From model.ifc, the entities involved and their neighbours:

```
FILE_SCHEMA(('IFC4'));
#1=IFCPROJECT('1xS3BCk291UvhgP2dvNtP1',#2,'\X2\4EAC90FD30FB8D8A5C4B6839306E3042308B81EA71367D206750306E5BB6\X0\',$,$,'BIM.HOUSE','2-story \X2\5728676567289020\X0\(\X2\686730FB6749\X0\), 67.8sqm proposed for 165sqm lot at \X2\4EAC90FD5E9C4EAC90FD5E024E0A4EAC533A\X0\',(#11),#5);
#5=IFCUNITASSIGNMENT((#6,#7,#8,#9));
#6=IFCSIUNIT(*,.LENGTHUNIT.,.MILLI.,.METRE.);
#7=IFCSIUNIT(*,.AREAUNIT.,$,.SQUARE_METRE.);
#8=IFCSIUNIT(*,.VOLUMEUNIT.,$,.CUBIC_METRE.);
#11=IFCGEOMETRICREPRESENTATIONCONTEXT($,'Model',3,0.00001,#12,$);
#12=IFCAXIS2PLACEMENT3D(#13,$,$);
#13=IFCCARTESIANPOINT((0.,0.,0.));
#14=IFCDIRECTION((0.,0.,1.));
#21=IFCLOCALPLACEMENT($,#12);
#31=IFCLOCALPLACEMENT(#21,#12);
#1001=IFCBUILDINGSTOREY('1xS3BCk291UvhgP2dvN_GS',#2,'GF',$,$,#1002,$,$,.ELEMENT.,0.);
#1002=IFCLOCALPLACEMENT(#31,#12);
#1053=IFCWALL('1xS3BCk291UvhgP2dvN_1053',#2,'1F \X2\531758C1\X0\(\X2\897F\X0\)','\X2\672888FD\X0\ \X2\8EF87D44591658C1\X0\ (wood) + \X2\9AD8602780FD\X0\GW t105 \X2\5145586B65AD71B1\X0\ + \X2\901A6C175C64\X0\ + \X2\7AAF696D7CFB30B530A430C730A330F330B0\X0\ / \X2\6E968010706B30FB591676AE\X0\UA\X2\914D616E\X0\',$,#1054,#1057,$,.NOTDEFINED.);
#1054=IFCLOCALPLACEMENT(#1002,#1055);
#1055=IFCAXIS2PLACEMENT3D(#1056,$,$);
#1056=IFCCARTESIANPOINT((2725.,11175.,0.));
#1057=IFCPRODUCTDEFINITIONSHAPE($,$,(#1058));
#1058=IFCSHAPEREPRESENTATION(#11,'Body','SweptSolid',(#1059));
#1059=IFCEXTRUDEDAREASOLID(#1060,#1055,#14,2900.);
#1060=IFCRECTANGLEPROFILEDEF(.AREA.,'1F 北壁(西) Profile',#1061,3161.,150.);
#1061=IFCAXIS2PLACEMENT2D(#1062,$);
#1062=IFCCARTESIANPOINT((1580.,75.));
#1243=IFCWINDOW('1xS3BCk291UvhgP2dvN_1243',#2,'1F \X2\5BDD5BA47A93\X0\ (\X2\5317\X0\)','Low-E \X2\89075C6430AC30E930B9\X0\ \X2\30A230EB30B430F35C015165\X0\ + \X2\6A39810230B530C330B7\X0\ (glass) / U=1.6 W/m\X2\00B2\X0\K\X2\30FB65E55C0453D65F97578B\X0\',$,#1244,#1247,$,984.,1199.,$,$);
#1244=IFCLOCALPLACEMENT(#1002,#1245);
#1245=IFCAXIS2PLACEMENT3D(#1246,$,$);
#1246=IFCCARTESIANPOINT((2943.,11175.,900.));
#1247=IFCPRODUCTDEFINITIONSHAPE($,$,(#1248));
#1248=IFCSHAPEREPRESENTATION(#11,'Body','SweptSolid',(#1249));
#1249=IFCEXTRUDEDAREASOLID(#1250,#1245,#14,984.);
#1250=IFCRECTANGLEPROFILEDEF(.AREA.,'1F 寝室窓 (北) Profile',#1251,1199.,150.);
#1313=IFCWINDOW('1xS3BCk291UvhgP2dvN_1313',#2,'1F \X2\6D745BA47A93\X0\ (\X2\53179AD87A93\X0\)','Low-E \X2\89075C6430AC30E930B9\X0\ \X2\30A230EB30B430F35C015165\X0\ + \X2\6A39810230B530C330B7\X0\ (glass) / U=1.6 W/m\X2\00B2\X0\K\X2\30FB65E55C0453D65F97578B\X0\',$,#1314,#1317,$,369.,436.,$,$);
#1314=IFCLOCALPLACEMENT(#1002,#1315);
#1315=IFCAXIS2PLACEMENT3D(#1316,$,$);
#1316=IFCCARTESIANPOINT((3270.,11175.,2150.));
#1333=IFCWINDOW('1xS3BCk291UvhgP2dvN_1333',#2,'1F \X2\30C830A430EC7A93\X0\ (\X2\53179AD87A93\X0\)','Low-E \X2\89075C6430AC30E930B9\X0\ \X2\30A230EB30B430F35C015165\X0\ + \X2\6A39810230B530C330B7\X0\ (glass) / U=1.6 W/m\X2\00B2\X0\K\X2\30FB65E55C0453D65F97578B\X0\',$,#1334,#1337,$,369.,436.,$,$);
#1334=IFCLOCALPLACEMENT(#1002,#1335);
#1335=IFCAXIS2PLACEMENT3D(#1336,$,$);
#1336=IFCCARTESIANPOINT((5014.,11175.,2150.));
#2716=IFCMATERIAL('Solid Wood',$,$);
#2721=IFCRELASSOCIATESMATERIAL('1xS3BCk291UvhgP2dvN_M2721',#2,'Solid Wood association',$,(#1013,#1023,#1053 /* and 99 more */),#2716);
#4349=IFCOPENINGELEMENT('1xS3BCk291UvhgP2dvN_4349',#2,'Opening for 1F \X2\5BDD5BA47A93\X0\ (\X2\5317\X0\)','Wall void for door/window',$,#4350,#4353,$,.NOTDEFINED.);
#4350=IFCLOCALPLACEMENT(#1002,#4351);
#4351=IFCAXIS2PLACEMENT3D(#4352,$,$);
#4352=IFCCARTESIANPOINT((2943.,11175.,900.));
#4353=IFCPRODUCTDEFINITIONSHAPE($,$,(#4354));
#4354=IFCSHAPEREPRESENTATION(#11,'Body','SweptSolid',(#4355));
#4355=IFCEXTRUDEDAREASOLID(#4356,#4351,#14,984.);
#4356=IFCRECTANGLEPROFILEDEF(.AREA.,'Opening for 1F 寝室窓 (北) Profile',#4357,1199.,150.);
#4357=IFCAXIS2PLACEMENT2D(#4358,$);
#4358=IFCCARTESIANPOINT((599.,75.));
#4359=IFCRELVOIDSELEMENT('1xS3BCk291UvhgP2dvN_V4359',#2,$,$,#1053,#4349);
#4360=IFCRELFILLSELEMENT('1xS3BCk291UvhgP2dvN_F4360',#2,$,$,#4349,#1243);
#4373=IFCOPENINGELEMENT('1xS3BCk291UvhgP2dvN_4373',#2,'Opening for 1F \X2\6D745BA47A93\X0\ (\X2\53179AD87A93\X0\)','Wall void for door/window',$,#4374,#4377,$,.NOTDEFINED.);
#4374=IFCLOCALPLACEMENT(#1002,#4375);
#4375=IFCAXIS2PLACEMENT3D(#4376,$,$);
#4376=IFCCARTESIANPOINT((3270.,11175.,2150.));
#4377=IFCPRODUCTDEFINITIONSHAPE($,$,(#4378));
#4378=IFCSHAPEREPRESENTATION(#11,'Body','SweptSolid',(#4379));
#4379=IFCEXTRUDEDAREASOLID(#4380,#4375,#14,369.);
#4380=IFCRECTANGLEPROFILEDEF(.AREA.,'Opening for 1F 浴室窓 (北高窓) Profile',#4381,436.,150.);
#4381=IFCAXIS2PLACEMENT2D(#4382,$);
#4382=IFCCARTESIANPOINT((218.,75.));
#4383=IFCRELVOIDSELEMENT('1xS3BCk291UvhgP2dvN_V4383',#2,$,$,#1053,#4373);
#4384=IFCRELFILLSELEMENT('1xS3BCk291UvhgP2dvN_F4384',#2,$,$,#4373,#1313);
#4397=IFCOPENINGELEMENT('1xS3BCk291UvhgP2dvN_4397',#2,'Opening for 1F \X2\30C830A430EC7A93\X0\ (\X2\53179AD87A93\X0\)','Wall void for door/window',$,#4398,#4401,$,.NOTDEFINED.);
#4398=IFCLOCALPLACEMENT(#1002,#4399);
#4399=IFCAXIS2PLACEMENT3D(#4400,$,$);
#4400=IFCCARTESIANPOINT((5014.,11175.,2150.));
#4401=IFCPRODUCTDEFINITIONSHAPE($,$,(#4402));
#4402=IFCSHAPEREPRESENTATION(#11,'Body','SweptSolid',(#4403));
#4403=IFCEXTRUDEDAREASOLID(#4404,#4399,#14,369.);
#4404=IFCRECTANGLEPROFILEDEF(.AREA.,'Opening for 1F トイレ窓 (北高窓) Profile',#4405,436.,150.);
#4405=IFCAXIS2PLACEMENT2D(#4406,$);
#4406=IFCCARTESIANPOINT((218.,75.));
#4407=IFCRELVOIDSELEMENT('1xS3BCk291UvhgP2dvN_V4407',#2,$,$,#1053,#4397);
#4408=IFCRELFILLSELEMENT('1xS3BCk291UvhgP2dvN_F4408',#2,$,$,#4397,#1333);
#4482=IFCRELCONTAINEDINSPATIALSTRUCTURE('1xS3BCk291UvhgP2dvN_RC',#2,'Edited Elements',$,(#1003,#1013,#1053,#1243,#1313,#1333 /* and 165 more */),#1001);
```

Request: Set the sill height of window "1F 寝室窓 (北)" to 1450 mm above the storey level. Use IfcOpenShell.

```python
import numpy as np
import ifcopenshell
import ifcopenshell.api.geometry
import ifcopenshell.geom
import ifcopenshell.util.element
import ifcopenshell.util.placement
import ifcopenshell.util.shape
import ifcopenshell.util.unit

model = ifcopenshell.open("model.ifc")
unit_scale = ifcopenshell.util.unit.calculate_unit_scale(model)

window = model.by_guid("1xS3BCk291UvhgP2dvN_1243")
opening = window.FillsVoids[0].RelatingOpeningElement
storey = ifcopenshell.util.element.get_container(window, ifc_class="IfcBuildingStorey")
level = ifcopenshell.util.placement.get_local_placement(storey.ObjectPlacement)[2, 3]

# The opening's origin need not be at the sill, so measure its lowest point.
shape = ifcopenshell.geom.create_shape(ifcopenshell.geom.settings(), opening)
bottom = ifcopenshell.util.shape.get_shape_bottom_elevation(shape, shape.geometry) / unit_scale
dz = level + 1.45 / unit_scale - bottom

shift = np.array([0.0, 0.0, dz])
# The window is not placed relative to its opening, so move both.
for product in (opening, window):
    matrix = ifcopenshell.util.placement.get_local_placement(product.ObjectPlacement)
    matrix[:3, 3] += shift
    ifcopenshell.api.geometry.edit_object_placement(model, product=product, matrix=matrix, is_si=False)

print(f"moved by {dz * unit_scale:+.3f} m")

model.write("model_rev.ifc")
```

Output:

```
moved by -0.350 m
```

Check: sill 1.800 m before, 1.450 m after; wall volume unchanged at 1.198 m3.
